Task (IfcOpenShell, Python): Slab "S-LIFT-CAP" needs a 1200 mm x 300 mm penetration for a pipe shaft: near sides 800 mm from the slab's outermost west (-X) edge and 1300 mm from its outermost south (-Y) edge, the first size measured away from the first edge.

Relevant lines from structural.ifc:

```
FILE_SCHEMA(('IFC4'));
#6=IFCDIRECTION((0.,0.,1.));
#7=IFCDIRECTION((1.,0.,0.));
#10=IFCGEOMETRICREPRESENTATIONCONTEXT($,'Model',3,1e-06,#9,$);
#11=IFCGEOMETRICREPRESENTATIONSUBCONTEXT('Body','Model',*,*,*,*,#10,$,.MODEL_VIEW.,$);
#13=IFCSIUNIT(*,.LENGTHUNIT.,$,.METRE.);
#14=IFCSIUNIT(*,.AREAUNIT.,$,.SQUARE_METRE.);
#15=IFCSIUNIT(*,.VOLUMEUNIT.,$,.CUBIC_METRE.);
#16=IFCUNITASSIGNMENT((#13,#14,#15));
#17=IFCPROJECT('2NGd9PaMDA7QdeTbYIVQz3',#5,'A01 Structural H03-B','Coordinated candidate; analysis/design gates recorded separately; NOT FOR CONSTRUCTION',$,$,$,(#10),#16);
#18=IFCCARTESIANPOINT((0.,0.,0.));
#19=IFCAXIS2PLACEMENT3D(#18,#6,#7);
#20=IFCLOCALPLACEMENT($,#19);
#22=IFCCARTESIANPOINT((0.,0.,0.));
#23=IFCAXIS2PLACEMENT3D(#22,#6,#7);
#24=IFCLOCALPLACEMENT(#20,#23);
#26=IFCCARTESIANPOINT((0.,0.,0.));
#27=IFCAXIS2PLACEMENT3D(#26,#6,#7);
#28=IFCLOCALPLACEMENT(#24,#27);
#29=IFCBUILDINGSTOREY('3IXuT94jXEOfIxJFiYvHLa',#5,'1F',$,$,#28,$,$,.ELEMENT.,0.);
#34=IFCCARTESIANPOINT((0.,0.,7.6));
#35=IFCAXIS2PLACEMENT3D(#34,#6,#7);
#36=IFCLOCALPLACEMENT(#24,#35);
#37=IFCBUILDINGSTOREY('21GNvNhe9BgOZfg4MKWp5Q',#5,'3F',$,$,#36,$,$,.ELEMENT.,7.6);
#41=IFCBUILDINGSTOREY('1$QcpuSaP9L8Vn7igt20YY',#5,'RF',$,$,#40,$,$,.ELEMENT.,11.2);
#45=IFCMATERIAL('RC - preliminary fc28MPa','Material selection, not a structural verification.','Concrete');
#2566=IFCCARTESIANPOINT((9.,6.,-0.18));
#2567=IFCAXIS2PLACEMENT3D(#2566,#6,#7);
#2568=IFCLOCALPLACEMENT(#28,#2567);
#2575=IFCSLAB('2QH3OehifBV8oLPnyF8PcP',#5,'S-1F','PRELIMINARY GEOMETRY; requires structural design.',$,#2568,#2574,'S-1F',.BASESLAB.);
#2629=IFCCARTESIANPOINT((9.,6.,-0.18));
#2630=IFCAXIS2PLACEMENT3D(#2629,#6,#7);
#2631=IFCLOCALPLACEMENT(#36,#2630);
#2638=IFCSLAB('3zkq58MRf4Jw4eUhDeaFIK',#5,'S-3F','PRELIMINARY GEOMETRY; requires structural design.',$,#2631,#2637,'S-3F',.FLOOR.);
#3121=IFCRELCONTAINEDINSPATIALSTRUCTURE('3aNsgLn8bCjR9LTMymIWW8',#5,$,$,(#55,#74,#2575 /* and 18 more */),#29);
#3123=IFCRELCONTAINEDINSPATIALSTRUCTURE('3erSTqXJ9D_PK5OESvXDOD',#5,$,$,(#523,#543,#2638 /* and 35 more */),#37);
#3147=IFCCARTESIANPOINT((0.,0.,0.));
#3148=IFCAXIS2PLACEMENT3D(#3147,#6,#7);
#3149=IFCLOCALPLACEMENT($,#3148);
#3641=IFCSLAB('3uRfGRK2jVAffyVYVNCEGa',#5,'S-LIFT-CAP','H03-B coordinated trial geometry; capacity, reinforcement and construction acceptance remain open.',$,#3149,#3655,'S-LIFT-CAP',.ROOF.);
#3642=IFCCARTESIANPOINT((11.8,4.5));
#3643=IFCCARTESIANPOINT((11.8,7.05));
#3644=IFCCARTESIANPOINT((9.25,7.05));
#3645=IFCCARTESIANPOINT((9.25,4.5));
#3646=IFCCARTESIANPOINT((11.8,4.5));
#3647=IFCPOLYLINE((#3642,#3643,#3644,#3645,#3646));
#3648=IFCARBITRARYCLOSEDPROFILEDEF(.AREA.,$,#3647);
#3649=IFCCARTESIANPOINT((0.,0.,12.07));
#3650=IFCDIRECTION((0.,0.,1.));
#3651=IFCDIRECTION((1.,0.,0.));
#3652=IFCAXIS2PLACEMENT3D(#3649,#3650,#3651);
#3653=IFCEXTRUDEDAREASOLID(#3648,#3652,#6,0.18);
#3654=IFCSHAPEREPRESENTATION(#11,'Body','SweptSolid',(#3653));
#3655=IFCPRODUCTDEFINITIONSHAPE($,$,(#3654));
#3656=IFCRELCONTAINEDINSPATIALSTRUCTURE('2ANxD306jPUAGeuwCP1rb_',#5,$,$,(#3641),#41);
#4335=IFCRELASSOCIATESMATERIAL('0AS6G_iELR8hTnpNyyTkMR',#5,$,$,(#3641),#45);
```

```python
import numpy as np
import ifcopenshell
import ifcopenshell.api.feature
import ifcopenshell.api.geometry
import ifcopenshell.api.root
import ifcopenshell.geom
import ifcopenshell.util.placement
import ifcopenshell.util.representation
import ifcopenshell.util.shape
import ifcopenshell.util.unit

model = ifcopenshell.open("structural.ifc")
unit_scale = ifcopenshell.util.unit.calculate_unit_scale(model)
settings = ifcopenshell.geom.settings()


def volume(element):
    """Net volume in cubic metres, openings subtracted."""
    shape = ifcopenshell.geom.create_shape(settings, element)
    return ifcopenshell.util.shape.get_volume(shape.geometry)


slab = model.by_guid("3uRfGRK2jVAffyVYVNCEGa")
before = volume(slab)

# Extent in the slab's own axes, in metres. The edges named are its -X and -Y sides.
slab_shape = ifcopenshell.geom.create_shape(settings, slab)
vertices = ifcopenshell.util.shape.get_vertices(slab_shape.geometry)
x_min, y_min, bottom = vertices.min(axis=0)
top = vertices[:, 2].max()

opening = ifcopenshell.api.root.create_entity(model, ifc_class="IfcOpeningElement", name="Pipe shaft opening", predefined_type="OPENING")
context = ifcopenshell.util.representation.get_context(model, "Model", "Body", "MODEL_VIEW")
width, depth = 1.2, 0.3
outline = [(0.0, 0.0), (width, 0.0), (width, depth), (0.0, depth), (0.0, 0.0)]
# Overshoot both faces by 50 mm so the cut is clean.
shape = ifcopenshell.api.geometry.add_slab_representation(
    model, context=context, depth=top - bottom + 0.1, polyline=outline
)
ifcopenshell.api.geometry.assign_representation(model, product=opening, representation=shape)

matrix = ifcopenshell.util.placement.get_local_placement(slab.ObjectPlacement)
matrix[:, 3] = matrix @ np.append(np.array([x_min + 0.8, y_min + 1.3, bottom - 0.05]) / unit_scale, 1.0)
ifcopenshell.api.geometry.edit_object_placement(model, product=opening, matrix=matrix, is_si=False)
ifcopenshell.api.feature.add_feature(model, feature=opening, element=slab)

after = volume(slab)

print(f"slab volume {before:.3f} -> {after:.3f} m3")

model.write("structural_rev.ifc")
```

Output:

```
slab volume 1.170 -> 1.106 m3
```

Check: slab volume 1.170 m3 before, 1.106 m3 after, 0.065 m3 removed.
